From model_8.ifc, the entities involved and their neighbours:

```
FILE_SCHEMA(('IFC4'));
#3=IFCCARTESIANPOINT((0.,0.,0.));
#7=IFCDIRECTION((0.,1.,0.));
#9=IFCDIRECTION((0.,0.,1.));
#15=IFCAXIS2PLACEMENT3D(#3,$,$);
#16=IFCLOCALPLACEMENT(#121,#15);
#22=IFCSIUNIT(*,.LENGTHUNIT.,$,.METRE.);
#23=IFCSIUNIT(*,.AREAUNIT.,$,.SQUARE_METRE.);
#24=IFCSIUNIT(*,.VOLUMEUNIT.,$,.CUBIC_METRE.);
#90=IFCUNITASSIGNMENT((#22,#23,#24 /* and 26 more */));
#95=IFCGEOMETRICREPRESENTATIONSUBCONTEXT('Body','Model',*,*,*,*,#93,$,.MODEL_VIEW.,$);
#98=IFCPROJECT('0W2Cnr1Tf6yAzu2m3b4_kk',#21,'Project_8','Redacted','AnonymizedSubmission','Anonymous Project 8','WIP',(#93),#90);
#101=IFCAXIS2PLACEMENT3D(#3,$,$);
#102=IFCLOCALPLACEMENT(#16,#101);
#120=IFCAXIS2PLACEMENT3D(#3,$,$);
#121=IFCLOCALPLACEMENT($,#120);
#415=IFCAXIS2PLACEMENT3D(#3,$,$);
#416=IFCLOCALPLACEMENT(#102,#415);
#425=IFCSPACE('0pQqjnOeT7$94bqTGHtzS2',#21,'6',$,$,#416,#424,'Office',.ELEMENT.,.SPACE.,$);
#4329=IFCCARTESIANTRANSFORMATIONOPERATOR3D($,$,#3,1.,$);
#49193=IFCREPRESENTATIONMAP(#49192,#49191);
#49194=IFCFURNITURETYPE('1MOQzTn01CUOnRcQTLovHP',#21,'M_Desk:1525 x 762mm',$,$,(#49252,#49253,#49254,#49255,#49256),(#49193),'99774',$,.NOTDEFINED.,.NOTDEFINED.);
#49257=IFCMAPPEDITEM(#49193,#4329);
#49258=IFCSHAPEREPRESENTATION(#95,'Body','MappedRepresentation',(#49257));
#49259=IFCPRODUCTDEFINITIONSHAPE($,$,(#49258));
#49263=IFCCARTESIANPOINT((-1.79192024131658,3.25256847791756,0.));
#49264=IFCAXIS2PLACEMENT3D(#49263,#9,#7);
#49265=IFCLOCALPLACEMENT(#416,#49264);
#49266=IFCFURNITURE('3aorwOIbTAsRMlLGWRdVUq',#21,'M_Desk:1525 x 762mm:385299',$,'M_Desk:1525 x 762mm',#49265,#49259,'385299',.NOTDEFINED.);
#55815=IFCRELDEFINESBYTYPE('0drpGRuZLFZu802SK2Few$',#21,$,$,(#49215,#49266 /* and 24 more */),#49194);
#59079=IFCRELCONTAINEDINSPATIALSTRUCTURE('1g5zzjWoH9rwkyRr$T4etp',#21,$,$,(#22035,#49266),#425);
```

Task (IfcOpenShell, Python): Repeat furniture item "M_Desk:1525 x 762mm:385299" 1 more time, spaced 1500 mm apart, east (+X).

```python
import numpy as np
import ifcopenshell
import ifcopenshell.api.geometry
import ifcopenshell.api.root
import ifcopenshell.util.element
import ifcopenshell.util.placement
import ifcopenshell.util.unit

model = ifcopenshell.open("model_8.ifc")
unit_scale = ifcopenshell.util.unit.calculate_unit_scale(model)


def reuse_history(source, copy):
    """copy_class also copies each property set's owner history, people and application; keep the originals."""
    for rel in copy.IsDefinedBy:
        if rel.is_a("IfcRelDefinesByProperties") and (history := rel.RelatingPropertyDefinition.OwnerHistory):
            rel.RelatingPropertyDefinition.OwnerHistory = source.OwnerHistory
            ifcopenshell.util.element.remove_deep2(model, history)


source = model.by_guid("3aorwOIbTAsRMlLGWRdVUq")
base = ifcopenshell.util.placement.get_local_placement(source.ObjectPlacement)
step = np.array([1.0, 0.0, 0.0]) * 1.5 / unit_scale

for i in range(1, 2):
    copy = ifcopenshell.api.root.copy_class(model, product=source)
    copy.Representation = ifcopenshell.util.element.copy_deep(
        model, source.Representation, exclude=["IfcGeometricRepresentationContext", "IfcRepresentationMap"]
    )
    copy.Name = "M_Desk:1525 x 762mm"
    copy.Tag = None
    reuse_history(source, copy)
    matrix = base.copy()
    matrix[:3, 3] += i * step
    print("added at", matrix[:3, 3].round(3) + 0.0)
    ifcopenshell.api.geometry.edit_object_placement(model, product=copy, matrix=matrix, is_si=False)

model.write("model_8_v2.ifc")
```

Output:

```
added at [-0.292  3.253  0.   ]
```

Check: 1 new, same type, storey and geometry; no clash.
